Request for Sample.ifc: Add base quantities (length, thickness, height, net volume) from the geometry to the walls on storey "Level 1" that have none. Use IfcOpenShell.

First a look at what the model holds.

```python
import ifcopenshell
import ifcopenshell.util.element
import ifcopenshell.util.unit

model = ifcopenshell.open("Sample.ifc")
print(model.schema)
for unit_type in ("LENGTHUNIT", "AREAUNIT", "VOLUMEUNIT"):
    print(unit_type, ifcopenshell.util.unit.calculate_unit_scale(model, unit_type))
storey = next(s for s in model.by_type("IfcBuildingStorey") if s.Name == "Level 1")
walls = [e for e in ifcopenshell.util.element.get_decomposition(storey) if e.is_a("IfcWall")]
for e in sorted(walls, key=lambda e: e.id()):
    print(e.id(), e.is_a(), e.Name, list(ifcopenshell.util.element.get_psets(e, qtos_only=True)), sep=" | ")
```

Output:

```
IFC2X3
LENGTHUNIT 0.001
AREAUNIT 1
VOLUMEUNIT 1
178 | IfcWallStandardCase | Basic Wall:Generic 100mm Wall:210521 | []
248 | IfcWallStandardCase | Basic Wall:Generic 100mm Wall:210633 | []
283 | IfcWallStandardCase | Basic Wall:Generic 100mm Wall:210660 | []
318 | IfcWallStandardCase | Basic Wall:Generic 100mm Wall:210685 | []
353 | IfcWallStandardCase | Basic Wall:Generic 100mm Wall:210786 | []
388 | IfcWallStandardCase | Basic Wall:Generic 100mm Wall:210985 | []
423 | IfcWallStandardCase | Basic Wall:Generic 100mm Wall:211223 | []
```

```python
import ifcopenshell
import ifcopenshell.api.pset
import ifcopenshell.geom
import ifcopenshell.util.element
import ifcopenshell.util.shape
import ifcopenshell.util.unit

model = ifcopenshell.open("Sample.ifc")
unit_scale = ifcopenshell.util.unit.calculate_unit_scale(model)
volume_scale = ifcopenshell.util.unit.calculate_unit_scale(model, "VOLUMEUNIT")
settings = ifcopenshell.geom.settings()

storey = next(s for s in model.by_type("IfcBuildingStorey") if s.Name == "Level 1")
walls = [e for e in ifcopenshell.util.element.get_decomposition(storey) if e.is_a("IfcWall")]

for e in sorted(walls, key=lambda e: e.id()):
    if ifcopenshell.util.element.get_psets(e, qtos_only=True, should_inherit=False):
        continue
    # Geometry comes back in metres, in the element's own axes.
    shape = ifcopenshell.geom.create_shape(settings, e)
    values = {
        "Length": ifcopenshell.util.shape.get_x(shape.geometry) / unit_scale,
        "Width": ifcopenshell.util.shape.get_y(shape.geometry) / unit_scale,
        "Height": ifcopenshell.util.shape.get_z(shape.geometry) / unit_scale,
        "NetVolume": ifcopenshell.util.shape.get_volume(shape.geometry) / volume_scale,
    }
    qto = ifcopenshell.api.pset.add_qto(model, product=e, name="BaseQuantities")
    ifcopenshell.api.pset.edit_qto(model, qto=qto, properties=values)
    print(e.id(), {k: round(v, 3) for k, v in values.items()})

model.write("Sample_updated.ifc")
```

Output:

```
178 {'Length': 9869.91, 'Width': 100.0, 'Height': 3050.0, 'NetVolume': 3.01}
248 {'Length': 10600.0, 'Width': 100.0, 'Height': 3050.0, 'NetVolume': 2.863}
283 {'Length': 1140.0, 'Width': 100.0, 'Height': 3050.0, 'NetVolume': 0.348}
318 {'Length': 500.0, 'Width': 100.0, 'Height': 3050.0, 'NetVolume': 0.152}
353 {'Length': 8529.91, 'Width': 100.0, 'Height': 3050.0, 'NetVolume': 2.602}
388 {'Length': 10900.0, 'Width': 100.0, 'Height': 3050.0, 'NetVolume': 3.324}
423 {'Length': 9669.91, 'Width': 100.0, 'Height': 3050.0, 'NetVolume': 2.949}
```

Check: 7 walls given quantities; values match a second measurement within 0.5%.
